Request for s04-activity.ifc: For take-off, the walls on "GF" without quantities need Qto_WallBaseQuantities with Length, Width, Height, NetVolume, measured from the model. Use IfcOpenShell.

First a look at what the model holds.

```python
import ifcopenshell
import ifcopenshell.util.element
import ifcopenshell.util.unit

model = ifcopenshell.open("s04-activity.ifc")
print(model.schema)
for unit_type in ("LENGTHUNIT", "AREAUNIT", "VOLUMEUNIT"):
    print(unit_type, ifcopenshell.util.unit.calculate_unit_scale(model, unit_type))
storey = next(s for s in model.by_type("IfcBuildingStorey") if s.Name == "GF")
walls = [e for e in ifcopenshell.util.element.get_decomposition(storey) if e.is_a("IfcWall")]
for e in sorted(walls, key=lambda e: e.id()):
    print(e.id(), e.is_a(), e.Name, list(ifcopenshell.util.element.get_psets(e, qtos_only=True)), sep=" | ")
```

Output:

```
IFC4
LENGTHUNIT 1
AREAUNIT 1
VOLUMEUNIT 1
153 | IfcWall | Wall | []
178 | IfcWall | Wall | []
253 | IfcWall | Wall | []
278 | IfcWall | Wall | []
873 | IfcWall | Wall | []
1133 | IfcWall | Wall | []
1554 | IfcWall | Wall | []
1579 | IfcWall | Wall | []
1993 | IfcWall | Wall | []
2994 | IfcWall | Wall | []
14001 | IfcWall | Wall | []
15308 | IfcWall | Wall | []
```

```python
import ifcopenshell
import ifcopenshell.api.pset
import ifcopenshell.geom
import ifcopenshell.util.element
import ifcopenshell.util.shape
import ifcopenshell.util.unit

model = ifcopenshell.open("s04-activity.ifc")
unit_scale = ifcopenshell.util.unit.calculate_unit_scale(model)
volume_scale = ifcopenshell.util.unit.calculate_unit_scale(model, "VOLUMEUNIT")
settings = ifcopenshell.geom.settings()

storey = next(s for s in model.by_type("IfcBuildingStorey") if s.Name == "GF")
walls = [e for e in ifcopenshell.util.element.get_decomposition(storey) if e.is_a("IfcWall")]

for e in sorted(walls, key=lambda e: e.id()):
    if ifcopenshell.util.element.get_psets(e, qtos_only=True, should_inherit=False):
        continue
    # Geometry comes back in metres, in the element's own axes.
    shape = ifcopenshell.geom.create_shape(settings, e)
    values = {
        "Length": ifcopenshell.util.shape.get_x(shape.geometry) / unit_scale,
        "Width": ifcopenshell.util.shape.get_y(shape.geometry) / unit_scale,
        "Height": ifcopenshell.util.shape.get_z(shape.geometry) / unit_scale,
        "NetVolume": ifcopenshell.util.shape.get_volume(shape.geometry) / volume_scale,
    }
    qto = ifcopenshell.api.pset.add_qto(model, product=e, name="Qto_WallBaseQuantities")
    ifcopenshell.api.pset.edit_qto(model, qto=qto, properties=values)
    print(e.id(), {k: round(v, 3) for k, v in values.items()})

model.write("s04-activity_v2.ifc")
```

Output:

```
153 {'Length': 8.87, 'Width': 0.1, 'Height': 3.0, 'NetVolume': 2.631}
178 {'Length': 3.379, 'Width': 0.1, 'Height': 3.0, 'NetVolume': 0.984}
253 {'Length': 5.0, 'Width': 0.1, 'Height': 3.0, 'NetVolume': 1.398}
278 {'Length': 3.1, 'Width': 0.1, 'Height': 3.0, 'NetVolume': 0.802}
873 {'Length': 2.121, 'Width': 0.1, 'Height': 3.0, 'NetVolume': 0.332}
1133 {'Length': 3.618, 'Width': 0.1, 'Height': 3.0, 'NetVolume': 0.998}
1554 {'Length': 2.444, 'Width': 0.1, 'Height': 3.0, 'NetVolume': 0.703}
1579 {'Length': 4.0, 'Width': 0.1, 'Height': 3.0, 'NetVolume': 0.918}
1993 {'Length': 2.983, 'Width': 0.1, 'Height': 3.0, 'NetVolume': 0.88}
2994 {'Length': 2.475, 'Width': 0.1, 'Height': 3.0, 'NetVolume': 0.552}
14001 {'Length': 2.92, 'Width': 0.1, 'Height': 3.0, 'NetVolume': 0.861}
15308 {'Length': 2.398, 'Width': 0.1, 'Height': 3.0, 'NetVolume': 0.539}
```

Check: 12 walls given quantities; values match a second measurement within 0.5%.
